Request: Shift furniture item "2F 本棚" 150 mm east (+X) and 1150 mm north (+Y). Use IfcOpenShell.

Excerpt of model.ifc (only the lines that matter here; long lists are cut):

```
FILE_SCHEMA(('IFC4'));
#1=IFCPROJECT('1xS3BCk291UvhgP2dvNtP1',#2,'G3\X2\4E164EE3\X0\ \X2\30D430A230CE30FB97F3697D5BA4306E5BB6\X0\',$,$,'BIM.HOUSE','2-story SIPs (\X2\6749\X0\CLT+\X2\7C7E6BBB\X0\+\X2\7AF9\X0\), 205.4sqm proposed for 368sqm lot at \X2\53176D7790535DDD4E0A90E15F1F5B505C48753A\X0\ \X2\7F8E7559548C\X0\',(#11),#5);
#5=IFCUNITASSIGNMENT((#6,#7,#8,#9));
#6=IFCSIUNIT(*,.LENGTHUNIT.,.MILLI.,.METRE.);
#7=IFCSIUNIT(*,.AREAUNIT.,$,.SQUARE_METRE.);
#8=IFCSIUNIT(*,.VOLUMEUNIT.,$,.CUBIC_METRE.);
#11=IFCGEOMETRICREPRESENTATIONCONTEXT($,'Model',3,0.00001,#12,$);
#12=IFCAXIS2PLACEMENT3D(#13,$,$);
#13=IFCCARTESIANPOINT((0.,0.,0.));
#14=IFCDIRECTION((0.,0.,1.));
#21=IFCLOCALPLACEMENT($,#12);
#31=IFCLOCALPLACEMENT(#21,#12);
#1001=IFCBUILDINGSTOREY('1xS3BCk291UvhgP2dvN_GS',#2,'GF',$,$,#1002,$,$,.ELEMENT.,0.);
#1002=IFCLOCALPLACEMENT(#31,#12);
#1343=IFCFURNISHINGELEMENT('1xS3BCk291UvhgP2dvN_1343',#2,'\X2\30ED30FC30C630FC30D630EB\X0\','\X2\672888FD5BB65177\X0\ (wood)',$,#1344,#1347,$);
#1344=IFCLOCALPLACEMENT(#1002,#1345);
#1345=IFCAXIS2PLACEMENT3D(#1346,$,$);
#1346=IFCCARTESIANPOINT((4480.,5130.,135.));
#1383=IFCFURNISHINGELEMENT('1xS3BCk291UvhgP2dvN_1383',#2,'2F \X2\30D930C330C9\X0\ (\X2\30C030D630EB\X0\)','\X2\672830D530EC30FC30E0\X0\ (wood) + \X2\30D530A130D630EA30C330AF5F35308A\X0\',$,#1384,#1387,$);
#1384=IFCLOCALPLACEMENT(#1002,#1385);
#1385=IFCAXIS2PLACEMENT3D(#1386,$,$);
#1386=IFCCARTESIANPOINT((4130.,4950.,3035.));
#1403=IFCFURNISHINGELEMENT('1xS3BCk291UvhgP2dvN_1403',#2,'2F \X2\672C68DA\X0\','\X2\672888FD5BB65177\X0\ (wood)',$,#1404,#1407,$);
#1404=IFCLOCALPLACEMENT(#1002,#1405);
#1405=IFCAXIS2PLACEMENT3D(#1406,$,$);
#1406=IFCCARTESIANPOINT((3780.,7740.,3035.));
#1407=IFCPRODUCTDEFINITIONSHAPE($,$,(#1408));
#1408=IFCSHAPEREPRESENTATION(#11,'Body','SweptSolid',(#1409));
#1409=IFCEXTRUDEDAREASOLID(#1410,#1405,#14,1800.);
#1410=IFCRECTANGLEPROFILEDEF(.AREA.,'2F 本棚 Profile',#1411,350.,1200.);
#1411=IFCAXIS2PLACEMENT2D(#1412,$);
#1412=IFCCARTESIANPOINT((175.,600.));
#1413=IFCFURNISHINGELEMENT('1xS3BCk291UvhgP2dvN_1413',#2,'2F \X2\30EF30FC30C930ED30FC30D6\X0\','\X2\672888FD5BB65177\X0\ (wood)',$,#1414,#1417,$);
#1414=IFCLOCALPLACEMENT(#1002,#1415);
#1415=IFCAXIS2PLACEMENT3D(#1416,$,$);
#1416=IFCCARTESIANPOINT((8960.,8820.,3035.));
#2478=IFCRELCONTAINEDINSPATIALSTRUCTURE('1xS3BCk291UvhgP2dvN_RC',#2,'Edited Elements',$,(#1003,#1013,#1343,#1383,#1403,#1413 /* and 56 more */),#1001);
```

```python
import ifcopenshell
import ifcopenshell.api.geometry
import ifcopenshell.util.placement
import ifcopenshell.util.unit

model = ifcopenshell.open("model.ifc")
unit_scale = ifcopenshell.util.unit.calculate_unit_scale(model)

item = model.by_guid("1xS3BCk291UvhgP2dvN_1403")
matrix = ifcopenshell.util.placement.get_local_placement(item.ObjectPlacement)
matrix[0, 3] += 0.15 / unit_scale
matrix[1, 3] += 1.15 / unit_scale
ifcopenshell.api.geometry.edit_object_placement(model, product=item, matrix=matrix, is_si=False)

print(ifcopenshell.util.placement.get_local_placement(item.ObjectPlacement).round(3) + 0.0)

model.write("model_updated.ifc")
```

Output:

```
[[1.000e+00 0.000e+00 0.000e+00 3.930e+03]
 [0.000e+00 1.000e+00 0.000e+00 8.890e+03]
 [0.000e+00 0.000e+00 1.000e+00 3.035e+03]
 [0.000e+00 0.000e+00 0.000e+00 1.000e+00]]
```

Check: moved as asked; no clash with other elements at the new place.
